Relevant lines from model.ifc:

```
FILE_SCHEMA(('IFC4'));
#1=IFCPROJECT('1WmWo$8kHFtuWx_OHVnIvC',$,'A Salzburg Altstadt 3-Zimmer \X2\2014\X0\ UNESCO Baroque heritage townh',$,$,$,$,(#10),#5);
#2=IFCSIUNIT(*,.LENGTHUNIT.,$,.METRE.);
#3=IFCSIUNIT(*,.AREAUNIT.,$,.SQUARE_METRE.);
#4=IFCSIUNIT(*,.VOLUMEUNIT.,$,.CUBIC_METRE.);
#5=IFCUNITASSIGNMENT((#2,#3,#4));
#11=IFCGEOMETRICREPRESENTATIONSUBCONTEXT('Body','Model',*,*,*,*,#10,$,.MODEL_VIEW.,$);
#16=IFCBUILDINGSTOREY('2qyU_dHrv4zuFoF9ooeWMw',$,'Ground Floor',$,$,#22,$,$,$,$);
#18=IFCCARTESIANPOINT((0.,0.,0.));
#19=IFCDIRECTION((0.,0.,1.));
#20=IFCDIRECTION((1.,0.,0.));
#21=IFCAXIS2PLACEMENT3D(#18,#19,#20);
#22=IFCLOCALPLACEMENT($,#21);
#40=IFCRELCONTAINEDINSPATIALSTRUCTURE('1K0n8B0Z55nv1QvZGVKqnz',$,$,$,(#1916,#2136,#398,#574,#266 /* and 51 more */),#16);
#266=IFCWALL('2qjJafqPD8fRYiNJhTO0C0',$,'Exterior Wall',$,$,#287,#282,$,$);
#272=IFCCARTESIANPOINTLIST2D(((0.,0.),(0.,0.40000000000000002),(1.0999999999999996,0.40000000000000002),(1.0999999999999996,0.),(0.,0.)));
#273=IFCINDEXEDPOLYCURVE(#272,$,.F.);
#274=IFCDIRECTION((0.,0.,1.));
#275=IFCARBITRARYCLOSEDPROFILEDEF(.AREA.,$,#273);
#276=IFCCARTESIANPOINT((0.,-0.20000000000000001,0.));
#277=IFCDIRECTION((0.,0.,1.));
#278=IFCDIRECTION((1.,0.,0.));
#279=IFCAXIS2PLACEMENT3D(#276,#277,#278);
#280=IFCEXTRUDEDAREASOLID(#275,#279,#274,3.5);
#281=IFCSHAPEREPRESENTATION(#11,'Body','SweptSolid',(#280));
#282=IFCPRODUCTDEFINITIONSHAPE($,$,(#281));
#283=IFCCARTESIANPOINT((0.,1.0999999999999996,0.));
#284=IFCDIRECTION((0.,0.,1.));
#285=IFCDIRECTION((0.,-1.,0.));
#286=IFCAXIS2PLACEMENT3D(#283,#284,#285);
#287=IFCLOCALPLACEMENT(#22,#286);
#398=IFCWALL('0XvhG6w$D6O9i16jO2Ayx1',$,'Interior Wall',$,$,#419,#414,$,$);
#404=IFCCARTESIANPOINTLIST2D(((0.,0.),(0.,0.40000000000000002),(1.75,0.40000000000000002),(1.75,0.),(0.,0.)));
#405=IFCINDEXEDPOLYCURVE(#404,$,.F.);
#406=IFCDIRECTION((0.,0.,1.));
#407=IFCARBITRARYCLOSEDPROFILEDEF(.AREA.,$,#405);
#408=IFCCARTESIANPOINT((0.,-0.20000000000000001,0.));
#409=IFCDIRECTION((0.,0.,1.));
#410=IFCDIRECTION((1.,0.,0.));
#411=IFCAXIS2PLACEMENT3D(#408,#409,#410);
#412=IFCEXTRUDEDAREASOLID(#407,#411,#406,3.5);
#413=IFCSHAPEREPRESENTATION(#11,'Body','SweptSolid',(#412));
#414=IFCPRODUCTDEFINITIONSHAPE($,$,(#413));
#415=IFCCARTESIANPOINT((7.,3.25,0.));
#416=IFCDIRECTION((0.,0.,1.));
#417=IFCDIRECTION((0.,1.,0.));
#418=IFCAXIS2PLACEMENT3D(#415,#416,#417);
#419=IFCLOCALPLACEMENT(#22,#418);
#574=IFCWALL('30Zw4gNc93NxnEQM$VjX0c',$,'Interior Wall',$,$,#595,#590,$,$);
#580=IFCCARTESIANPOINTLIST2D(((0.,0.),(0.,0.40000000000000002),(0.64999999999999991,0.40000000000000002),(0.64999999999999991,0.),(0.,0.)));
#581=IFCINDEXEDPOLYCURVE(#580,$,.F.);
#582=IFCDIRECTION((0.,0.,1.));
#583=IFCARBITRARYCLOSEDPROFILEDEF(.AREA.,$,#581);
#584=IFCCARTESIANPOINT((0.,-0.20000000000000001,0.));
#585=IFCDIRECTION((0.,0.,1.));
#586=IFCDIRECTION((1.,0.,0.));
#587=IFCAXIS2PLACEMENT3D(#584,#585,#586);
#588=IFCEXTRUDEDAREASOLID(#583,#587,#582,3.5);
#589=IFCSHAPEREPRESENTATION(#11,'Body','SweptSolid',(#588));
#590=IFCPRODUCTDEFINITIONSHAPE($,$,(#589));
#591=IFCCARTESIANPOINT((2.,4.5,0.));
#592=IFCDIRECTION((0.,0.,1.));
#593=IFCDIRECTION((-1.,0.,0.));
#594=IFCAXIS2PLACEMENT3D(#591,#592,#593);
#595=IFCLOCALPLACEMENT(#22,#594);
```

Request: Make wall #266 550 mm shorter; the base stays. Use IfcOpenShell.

```python
import ifcopenshell
import ifcopenshell.geom
import ifcopenshell.util.representation
import ifcopenshell.util.shape
import ifcopenshell.util.unit

model = ifcopenshell.open("model.ifc")
unit_scale = ifcopenshell.util.unit.calculate_unit_scale(model)
settings = ifcopenshell.geom.settings()


def volume(element):
    """Net volume in cubic metres, openings subtracted."""
    shape = ifcopenshell.geom.create_shape(settings, element)
    return ifcopenshell.util.shape.get_volume(shape.geometry)


wall = model.by_guid("2qjJafqPD8fRYiNJhTO0C0")
before = volume(wall)

body = ifcopenshell.util.representation.get_representation(wall, "Model", "Body")
solid = body.Items[0]
old_height = solid.Depth
solid.Depth -= 0.55 / unit_scale
after = volume(wall)

print(f"height {old_height:g} -> {solid.Depth:g}, volume {before:.3f} -> {after:.3f} m3")

model.write("model_v2.ifc")
```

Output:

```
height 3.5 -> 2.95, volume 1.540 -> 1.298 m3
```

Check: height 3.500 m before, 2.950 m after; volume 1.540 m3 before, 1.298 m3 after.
